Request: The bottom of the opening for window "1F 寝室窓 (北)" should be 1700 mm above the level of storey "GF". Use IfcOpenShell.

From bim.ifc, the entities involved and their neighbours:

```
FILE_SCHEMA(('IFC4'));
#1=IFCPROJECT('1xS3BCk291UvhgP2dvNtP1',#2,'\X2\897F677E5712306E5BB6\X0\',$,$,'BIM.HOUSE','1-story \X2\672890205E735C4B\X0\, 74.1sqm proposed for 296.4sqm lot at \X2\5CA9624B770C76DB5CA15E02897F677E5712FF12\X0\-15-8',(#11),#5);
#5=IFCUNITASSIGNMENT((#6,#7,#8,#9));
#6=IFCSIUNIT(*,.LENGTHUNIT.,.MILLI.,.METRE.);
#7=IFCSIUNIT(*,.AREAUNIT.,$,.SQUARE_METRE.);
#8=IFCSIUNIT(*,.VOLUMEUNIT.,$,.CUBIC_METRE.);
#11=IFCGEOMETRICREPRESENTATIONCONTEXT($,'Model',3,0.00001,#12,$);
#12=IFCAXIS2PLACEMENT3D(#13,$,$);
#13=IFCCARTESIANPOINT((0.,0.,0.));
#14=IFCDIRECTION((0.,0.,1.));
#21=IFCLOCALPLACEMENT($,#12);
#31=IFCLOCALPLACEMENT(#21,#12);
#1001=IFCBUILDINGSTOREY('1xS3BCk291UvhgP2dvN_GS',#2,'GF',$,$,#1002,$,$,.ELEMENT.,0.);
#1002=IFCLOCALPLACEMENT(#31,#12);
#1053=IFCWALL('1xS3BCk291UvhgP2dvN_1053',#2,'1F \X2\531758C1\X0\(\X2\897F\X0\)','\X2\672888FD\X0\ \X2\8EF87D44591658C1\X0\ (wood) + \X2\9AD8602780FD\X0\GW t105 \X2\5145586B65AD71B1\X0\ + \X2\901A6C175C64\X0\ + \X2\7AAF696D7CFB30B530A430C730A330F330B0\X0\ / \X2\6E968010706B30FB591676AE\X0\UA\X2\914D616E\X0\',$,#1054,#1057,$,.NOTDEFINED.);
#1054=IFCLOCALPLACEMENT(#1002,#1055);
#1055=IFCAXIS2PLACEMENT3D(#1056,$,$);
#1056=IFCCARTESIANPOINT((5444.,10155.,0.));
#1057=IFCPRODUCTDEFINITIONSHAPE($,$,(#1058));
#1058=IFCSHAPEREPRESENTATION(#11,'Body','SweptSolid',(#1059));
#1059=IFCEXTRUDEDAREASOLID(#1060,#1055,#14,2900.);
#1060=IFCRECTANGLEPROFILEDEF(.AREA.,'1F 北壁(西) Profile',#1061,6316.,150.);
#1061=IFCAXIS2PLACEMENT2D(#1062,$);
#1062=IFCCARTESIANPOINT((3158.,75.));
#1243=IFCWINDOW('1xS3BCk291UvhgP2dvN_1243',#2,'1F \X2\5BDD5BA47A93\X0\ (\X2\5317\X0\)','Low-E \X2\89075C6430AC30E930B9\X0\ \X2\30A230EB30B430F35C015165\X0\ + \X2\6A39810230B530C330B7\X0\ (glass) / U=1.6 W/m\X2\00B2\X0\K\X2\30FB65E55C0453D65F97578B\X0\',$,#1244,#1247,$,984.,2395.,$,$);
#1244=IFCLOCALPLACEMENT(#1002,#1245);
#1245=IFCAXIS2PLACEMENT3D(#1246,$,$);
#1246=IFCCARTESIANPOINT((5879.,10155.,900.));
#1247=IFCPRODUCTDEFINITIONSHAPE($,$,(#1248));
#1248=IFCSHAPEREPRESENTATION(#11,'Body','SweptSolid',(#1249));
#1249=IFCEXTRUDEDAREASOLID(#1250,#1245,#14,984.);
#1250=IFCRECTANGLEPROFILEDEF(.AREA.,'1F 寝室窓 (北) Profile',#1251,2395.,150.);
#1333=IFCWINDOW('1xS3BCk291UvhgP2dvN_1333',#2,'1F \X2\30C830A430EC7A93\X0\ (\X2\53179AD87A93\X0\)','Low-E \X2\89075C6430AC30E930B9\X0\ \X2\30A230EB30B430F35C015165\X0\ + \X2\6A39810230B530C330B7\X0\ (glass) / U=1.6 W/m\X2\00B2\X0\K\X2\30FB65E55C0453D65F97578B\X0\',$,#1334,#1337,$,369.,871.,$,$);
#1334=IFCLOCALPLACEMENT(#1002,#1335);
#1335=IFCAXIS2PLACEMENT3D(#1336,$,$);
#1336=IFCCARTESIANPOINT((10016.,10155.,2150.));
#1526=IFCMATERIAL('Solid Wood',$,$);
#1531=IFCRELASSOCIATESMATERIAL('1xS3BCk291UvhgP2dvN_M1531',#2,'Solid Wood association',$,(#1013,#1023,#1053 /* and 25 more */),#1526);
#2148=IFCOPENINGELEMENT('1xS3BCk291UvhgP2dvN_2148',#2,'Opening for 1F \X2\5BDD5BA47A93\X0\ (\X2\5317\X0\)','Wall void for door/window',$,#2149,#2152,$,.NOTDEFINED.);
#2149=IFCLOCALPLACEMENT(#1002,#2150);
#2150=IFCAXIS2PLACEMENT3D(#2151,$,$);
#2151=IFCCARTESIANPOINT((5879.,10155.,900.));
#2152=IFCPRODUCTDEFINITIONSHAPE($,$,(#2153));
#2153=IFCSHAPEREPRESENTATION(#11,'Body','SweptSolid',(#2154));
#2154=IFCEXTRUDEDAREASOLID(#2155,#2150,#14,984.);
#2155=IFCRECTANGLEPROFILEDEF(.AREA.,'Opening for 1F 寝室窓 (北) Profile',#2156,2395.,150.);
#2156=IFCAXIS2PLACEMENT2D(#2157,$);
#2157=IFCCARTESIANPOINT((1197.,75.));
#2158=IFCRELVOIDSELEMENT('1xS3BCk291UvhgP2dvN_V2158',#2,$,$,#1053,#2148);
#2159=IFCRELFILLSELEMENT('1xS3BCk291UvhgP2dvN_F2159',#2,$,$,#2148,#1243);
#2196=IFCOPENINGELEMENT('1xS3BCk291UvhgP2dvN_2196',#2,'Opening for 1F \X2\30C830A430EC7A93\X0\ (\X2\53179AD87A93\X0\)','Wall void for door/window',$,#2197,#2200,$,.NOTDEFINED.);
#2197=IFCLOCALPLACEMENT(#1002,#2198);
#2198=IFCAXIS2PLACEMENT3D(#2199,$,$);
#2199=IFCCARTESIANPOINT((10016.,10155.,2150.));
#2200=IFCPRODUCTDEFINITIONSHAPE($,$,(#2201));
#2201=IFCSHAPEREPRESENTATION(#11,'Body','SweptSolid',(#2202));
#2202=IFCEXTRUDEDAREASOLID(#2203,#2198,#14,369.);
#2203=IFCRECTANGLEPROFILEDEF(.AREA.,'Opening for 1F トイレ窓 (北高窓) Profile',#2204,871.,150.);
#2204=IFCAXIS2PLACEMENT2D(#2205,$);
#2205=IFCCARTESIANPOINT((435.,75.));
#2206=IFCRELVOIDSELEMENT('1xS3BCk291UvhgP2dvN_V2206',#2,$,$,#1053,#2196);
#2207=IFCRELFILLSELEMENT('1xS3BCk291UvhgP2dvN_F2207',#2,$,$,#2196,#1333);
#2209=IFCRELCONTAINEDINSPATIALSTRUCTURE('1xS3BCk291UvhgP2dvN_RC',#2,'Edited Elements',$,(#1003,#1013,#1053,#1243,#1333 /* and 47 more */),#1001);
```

```python
import numpy as np
import ifcopenshell
import ifcopenshell.api.geometry
import ifcopenshell.geom
import ifcopenshell.util.element
import ifcopenshell.util.placement
import ifcopenshell.util.shape
import ifcopenshell.util.unit

model = ifcopenshell.open("bim.ifc")
unit_scale = ifcopenshell.util.unit.calculate_unit_scale(model)

window = model.by_guid("1xS3BCk291UvhgP2dvN_1243")
opening = window.FillsVoids[0].RelatingOpeningElement
storey = ifcopenshell.util.element.get_container(window, ifc_class="IfcBuildingStorey")
level = ifcopenshell.util.placement.get_local_placement(storey.ObjectPlacement)[2, 3]

# The opening's origin need not be at the sill, so measure its lowest point.
shape = ifcopenshell.geom.create_shape(ifcopenshell.geom.settings(), opening)
bottom = ifcopenshell.util.shape.get_shape_bottom_elevation(shape, shape.geometry) / unit_scale
dz = level + 1.7 / unit_scale - bottom

shift = np.array([0.0, 0.0, dz])
# The window is not placed relative to its opening, so move both.
for product in (opening, window):
    matrix = ifcopenshell.util.placement.get_local_placement(product.ObjectPlacement)
    matrix[:3, 3] += shift
    ifcopenshell.api.geometry.edit_object_placement(model, product=product, matrix=matrix, is_si=False)

print(f"moved by {dz * unit_scale:+.3f} m")

model.write("bim_edited.ifc")
```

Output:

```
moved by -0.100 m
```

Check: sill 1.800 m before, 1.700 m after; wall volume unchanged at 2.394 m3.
